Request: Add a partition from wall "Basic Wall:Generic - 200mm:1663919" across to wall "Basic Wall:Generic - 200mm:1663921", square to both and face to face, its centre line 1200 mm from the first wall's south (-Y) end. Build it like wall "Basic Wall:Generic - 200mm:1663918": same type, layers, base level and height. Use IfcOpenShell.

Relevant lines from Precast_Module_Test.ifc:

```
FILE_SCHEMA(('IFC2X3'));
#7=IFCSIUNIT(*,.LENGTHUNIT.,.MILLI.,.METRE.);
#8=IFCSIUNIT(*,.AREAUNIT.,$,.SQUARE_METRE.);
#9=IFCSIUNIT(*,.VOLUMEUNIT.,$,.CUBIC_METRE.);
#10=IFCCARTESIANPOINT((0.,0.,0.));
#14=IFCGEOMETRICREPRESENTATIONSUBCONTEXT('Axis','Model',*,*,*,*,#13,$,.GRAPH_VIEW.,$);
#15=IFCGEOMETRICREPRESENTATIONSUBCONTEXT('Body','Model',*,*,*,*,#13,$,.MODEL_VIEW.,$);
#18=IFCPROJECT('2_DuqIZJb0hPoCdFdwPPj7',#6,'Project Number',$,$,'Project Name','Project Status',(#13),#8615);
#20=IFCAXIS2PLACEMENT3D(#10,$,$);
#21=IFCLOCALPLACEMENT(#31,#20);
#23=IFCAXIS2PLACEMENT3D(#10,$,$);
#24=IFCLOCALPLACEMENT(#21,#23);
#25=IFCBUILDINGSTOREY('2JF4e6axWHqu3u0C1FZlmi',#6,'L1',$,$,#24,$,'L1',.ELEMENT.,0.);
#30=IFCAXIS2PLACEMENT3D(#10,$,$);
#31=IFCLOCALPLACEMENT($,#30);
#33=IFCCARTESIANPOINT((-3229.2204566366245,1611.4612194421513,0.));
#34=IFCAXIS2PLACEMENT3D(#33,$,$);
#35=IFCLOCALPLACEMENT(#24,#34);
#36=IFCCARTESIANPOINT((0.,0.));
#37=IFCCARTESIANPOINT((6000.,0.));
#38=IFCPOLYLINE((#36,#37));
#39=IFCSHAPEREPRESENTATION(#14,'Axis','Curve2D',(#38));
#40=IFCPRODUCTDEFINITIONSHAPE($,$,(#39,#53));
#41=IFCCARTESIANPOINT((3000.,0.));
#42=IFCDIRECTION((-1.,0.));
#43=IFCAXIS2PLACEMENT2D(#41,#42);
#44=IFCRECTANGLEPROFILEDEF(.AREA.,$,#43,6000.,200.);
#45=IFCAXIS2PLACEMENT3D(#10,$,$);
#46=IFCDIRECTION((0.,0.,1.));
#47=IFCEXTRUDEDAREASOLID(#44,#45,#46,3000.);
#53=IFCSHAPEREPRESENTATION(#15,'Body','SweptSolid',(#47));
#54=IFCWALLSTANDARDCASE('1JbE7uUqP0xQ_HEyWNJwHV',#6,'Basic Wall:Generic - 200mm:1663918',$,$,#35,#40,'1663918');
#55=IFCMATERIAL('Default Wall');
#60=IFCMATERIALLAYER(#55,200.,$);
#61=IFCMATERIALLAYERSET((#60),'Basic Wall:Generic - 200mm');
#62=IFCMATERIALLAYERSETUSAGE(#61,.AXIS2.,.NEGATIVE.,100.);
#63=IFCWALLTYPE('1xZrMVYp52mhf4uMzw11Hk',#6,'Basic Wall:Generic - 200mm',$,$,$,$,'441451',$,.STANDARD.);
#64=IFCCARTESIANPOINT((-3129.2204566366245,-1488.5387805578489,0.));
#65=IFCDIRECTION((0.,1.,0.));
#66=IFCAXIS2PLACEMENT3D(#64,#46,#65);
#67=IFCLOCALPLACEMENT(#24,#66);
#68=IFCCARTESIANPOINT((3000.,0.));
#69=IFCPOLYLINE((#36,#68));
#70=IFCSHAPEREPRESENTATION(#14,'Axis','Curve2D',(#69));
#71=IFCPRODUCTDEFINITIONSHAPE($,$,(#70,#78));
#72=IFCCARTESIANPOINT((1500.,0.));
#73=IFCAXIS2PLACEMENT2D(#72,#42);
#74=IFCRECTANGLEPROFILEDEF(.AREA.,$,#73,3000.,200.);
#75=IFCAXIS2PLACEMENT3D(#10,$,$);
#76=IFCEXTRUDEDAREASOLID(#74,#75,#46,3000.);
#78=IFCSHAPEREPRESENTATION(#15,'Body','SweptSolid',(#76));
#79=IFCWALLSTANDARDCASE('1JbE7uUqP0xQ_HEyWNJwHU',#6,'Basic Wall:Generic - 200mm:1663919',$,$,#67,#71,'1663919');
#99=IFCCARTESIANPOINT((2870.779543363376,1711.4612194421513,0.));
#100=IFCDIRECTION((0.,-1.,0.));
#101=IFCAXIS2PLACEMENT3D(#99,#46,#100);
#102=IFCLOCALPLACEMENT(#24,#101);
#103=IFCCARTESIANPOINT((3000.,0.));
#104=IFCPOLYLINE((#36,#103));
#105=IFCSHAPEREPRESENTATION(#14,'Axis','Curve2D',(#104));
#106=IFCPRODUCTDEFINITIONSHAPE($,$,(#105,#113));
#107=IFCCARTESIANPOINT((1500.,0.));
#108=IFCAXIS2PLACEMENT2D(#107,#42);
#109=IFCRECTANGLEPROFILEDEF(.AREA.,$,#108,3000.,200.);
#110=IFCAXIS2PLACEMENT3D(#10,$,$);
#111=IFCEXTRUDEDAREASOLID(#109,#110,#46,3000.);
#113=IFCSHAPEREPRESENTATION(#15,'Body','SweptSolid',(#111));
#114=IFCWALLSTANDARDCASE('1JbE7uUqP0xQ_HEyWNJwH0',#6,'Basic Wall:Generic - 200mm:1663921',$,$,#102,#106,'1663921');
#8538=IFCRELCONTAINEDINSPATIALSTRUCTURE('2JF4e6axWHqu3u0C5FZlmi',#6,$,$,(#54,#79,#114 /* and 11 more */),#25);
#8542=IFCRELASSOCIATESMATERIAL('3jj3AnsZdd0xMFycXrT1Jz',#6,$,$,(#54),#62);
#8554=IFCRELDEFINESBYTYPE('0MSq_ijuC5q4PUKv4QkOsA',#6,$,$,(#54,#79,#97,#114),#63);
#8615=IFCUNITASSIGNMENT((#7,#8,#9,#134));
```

```python
import numpy as np
import ifcopenshell
import ifcopenshell.api.geometry
import ifcopenshell.api.material
import ifcopenshell.api.pset
import ifcopenshell.api.root
import ifcopenshell.api.spatial
import ifcopenshell.api.type
import ifcopenshell.geom
import ifcopenshell.util.element
import ifcopenshell.util.placement
import ifcopenshell.util.representation
import ifcopenshell.util.shape
import ifcopenshell.util.unit

model = ifcopenshell.open("Precast_Module_Test.ifc")
unit_scale = ifcopenshell.util.unit.calculate_unit_scale(model)
settings = ifcopenshell.geom.settings()
settings.set("use-world-coords", True)

start_wall = model.by_guid("1JbE7uUqP0xQ_HEyWNJwHU")
end_wall = model.by_id(114)
like = model.by_guid("1JbE7uUqP0xQ_HEyWNJwHV")
matrix = ifcopenshell.util.placement.get_local_placement(start_wall.ObjectPlacement)
matrix[:3, 3] *= unit_scale


def extent(element):
    """Bounding box in the first wall's axes, in metres."""
    shape = ifcopenshell.geom.create_shape(settings, element)
    points = (ifcopenshell.util.shape.get_vertices(shape.geometry) - matrix[:3, 3]) @ matrix[:3, :3]
    return points.min(axis=0), points.max(axis=0)


y_start = extent(start_wall)[0][1]
y_end = extent(end_wall)[1][1]
like_min, like_max = extent(like)
length, height = float(abs(y_end - y_start)), float(like_max[2] - like_min[2])
layer_set = ifcopenshell.util.element.get_material(like, should_skip_usage=True)
thickness = sum(layer.LayerThickness for layer in layer_set.MaterialLayers) * unit_scale

wall = ifcopenshell.api.root.create_entity(model, ifc_class="IfcWallStandardCase", name="New partition")
storey = ifcopenshell.util.element.get_container(like)
ifcopenshell.api.spatial.assign_container(model, products=[wall], relating_structure=storey)
ifcopenshell.api.type.assign_type(
    model, related_objects=[wall], relating_type=ifcopenshell.util.element.get_type(like), should_map_representations=False
)
rel = ifcopenshell.api.material.assign_material(
    model, products=[wall], type="IfcMaterialLayerSetUsage", material=layer_set
)
rel.RelatingMaterial.OffsetFromReferenceLine = -thickness / 2 / unit_scale
pset = ifcopenshell.api.pset.add_pset(model, product=wall, name="Pset_WallCommon")
ifcopenshell.api.pset.edit_pset(model, pset=pset, properties={"IsExternal": False, "LoadBearing": False})

# The axis runs down the middle of the wall.
axis = ifcopenshell.api.geometry.add_axis_representation(
    model, context=ifcopenshell.util.representation.get_context(model, "Model", "Axis"), axis=[(0.0, 0.0), (length, 0.0)]
)
body = ifcopenshell.api.geometry.add_wall_representation(
    model,
    context=ifcopenshell.util.representation.get_context(model, "Model", "Body", "MODEL_VIEW"),
    length=length,
    height=height,
    thickness=thickness,
    offset=-thickness / 2,
)
for representation in (axis, body):
    ifcopenshell.api.geometry.assign_representation(model, product=wall, representation=representation)

placement = matrix @ ifcopenshell.util.placement.rotation(-90, "Z")
placement[:, 3] = matrix @ np.array([extent(start_wall)[0][0] + 1.2, y_start, like_min[2], 1.0])
ifcopenshell.api.geometry.edit_object_placement(model, product=wall, matrix=placement)

print(f"partition {length:.3f} m long, {height:.3f} m high, {thickness:.3f} m thick")

model.write("Precast_Module_Test_edited.ifc")
```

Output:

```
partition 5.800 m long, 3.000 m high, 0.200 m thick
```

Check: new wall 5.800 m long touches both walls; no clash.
